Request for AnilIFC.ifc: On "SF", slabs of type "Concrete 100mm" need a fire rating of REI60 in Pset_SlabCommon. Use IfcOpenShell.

First a look at what the model holds.

```python
import ifcopenshell
import ifcopenshell.util.element

model = ifcopenshell.open("AnilIFC.ifc")
print(model.schema)
storey = next(s for s in model.by_type("IfcBuildingStorey") if s.Name == "SF")
slabs = [e for e in ifcopenshell.util.element.get_decomposition(storey) if e.is_a("IfcSlab")]
seen = {}
for e in slabs:
    element_type = ifcopenshell.util.element.get_type(e)
    key = (element_type.Name if element_type != e and element_type else None, ifcopenshell.util.element.get_pset(e, "Pset_SlabCommon", "FireRating"))
    seen[key] = seen.get(key, 0) + 1
for (name, value), count in sorted(seen.items(), key=str):
    print(count, "x", name, "|", value)
```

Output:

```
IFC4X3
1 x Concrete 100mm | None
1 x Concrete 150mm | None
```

```python
import ifcopenshell
import ifcopenshell.api.pset
import ifcopenshell.util.element

model = ifcopenshell.open("AnilIFC.ifc")

storey = next(s for s in model.by_type("IfcBuildingStorey") if s.Name == "SF")
slabs = [e for e in ifcopenshell.util.element.get_decomposition(storey) if e.is_a("IfcSlab")]

count = 0
for e in slabs:
    element_type = ifcopenshell.util.element.get_type(e)
    if element_type in (None, e) or element_type.Name != "Concrete 100mm":
        continue
    # add_pset returns the element's existing set when there is one.
    pset = ifcopenshell.api.pset.add_pset(model, product=e, name="Pset_SlabCommon")
    ifcopenshell.api.pset.edit_pset(model, pset=pset, properties={"FireRating": "REI60"})
    count += 1

print(count, "slabs updated")

model.write("AnilIFC_edited.ifc")
```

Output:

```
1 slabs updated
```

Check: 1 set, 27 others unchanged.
